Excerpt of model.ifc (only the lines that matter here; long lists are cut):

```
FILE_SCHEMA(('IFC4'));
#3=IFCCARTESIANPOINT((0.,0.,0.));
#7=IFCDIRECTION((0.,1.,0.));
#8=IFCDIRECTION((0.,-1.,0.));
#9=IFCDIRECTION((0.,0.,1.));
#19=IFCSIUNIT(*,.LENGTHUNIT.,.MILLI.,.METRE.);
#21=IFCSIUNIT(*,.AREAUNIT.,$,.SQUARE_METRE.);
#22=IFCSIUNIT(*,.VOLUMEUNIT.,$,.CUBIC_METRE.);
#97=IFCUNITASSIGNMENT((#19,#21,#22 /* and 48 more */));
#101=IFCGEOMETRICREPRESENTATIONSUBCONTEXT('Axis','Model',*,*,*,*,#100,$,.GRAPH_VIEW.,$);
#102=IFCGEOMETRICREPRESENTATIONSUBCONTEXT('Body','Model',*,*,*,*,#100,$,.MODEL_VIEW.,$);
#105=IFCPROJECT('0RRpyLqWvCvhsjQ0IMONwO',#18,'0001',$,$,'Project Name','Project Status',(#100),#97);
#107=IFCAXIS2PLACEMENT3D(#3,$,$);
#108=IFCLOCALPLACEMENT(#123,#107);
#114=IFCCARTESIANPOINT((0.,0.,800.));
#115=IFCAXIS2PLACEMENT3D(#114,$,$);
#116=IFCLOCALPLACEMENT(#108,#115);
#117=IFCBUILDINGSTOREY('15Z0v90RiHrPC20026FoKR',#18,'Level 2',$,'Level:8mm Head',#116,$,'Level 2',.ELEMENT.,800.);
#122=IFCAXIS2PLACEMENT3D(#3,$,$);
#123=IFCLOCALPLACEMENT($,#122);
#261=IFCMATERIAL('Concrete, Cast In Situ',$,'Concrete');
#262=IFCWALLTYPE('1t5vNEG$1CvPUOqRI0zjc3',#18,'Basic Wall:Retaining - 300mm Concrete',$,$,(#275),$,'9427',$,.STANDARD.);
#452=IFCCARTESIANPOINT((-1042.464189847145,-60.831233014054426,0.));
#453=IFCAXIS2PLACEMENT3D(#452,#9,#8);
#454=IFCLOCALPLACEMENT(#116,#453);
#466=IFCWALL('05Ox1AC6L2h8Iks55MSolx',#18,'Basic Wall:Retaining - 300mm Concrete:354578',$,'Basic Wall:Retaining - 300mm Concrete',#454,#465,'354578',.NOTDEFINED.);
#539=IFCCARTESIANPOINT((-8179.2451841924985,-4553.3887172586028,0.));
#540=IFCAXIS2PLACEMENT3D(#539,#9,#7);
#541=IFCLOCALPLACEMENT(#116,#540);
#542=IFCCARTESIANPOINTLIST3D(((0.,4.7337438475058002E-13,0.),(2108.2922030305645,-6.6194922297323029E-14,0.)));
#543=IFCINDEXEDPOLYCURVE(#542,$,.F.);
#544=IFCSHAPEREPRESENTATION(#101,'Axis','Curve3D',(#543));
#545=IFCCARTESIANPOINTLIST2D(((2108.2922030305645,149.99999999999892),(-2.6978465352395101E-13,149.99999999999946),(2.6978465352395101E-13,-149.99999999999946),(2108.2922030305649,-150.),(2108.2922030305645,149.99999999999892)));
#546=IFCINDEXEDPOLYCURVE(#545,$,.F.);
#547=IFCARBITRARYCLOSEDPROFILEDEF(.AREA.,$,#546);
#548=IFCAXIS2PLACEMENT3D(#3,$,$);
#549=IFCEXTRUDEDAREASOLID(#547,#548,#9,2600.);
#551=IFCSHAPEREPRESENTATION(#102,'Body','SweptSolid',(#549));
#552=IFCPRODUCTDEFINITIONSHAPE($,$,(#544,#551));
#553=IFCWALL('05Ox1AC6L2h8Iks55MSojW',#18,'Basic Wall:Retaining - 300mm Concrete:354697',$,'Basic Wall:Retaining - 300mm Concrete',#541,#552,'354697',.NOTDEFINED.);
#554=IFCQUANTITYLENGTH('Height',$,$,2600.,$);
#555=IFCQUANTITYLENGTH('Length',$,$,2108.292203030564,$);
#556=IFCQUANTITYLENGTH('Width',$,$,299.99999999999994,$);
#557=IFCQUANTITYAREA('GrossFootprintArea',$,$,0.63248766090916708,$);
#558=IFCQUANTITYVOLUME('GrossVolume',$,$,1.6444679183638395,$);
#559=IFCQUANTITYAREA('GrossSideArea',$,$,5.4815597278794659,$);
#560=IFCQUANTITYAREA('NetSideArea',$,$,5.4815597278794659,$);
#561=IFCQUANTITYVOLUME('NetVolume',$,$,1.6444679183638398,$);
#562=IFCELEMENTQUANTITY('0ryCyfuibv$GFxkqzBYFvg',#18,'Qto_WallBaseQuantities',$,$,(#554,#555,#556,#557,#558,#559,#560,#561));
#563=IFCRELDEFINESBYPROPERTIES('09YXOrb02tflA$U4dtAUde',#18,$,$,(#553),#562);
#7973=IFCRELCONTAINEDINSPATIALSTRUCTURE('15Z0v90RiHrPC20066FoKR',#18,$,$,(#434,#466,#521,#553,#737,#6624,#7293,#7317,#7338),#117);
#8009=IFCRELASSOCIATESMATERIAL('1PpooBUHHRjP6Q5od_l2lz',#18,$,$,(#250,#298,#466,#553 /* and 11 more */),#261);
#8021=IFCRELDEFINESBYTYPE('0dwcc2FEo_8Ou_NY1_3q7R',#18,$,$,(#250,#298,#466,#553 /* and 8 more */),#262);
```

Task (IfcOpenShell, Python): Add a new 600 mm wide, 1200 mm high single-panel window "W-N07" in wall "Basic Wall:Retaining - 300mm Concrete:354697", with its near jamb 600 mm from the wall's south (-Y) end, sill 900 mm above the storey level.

```python
import numpy as np
import ifcopenshell
import ifcopenshell.api.feature
import ifcopenshell.api.geometry
import ifcopenshell.api.pset
import ifcopenshell.api.root
import ifcopenshell.api.spatial
import ifcopenshell.geom
import ifcopenshell.util.element
import ifcopenshell.util.placement
import ifcopenshell.util.representation
import ifcopenshell.util.shape
import ifcopenshell.util.unit

model = ifcopenshell.open("model.ifc")
unit_scale = ifcopenshell.util.unit.calculate_unit_scale(model)
area_scale = ifcopenshell.util.unit.calculate_unit_scale(model, "AREAUNIT")
volume_scale = ifcopenshell.util.unit.calculate_unit_scale(model, "VOLUMEUNIT")
settings = ifcopenshell.geom.settings()


def volume(element):
    """Net volume in cubic metres, openings subtracted."""
    shape = ifcopenshell.geom.create_shape(settings, element)
    return ifcopenshell.util.shape.get_volume(shape.geometry)


wall = model.by_id(553)
storey = ifcopenshell.util.element.get_container(wall, ifc_class="IfcBuildingStorey")
context = ifcopenshell.util.representation.get_context(model, "Model", "Body", "MODEL_VIEW")
before = volume(wall)

width, height, from_end, sill = 0.6, 1.2, 0.6, 0.9  # metres

# The wall runs along its own X axis, and the end named is its -X end.
wall_shape = ifcopenshell.geom.create_shape(settings, wall)
x, y, z = ifcopenshell.util.shape.get_vertices(wall_shape.geometry).T
start = x.min() + from_end
face, thickness = float(y.min()), float(y.max() - y.min())
wall_matrix = ifcopenshell.util.placement.get_local_placement(wall.ObjectPlacement)
level = ifcopenshell.util.placement.get_local_placement(storey.ObjectPlacement)[2, 3]


def in_wall(x, y):
    """Placement at x, y metres in the wall's axes, at sill height."""
    matrix = wall_matrix.copy()
    matrix[:, 3] = wall_matrix @ np.array([x / unit_scale, y / unit_scale, 0.0, 1.0])
    matrix[2, 3] = level + sill / unit_scale
    return matrix


# Opening: a box that overshoots both wall faces by 50 mm.
opening = ifcopenshell.api.root.create_entity(model, ifc_class="IfcOpeningElement", predefined_type="OPENING")
box = ifcopenshell.api.geometry.add_wall_representation(
    model, context=context, length=width, height=height, thickness=thickness + 0.1
)
ifcopenshell.api.geometry.assign_representation(model, product=opening, representation=box)
ifcopenshell.api.geometry.edit_object_placement(model, product=opening, matrix=in_wall(start, face - 0.05), is_si=False)
ifcopenshell.api.feature.add_feature(model, feature=opening, element=wall)

window = ifcopenshell.api.root.create_entity(model, ifc_class="IfcWindow", name="W-N07", predefined_type="WINDOW")
window.OverallWidth, window.OverallHeight = width / unit_scale, height / unit_scale
window.PartitioningType = "SINGLE_PANEL"
body = ifcopenshell.api.geometry.add_window_representation(
    model,
    context=context,
    overall_width=window.OverallWidth,
    overall_height=window.OverallHeight,
    partition_type="SINGLE_PANEL",
)
ifcopenshell.api.geometry.assign_representation(model, product=window, representation=body)
ifcopenshell.api.spatial.assign_container(model, products=[window], relating_structure=storey)
ifcopenshell.api.feature.add_filling(model, opening=opening, element=window)

# Centre the window in the wall's thickness.
ifcopenshell.api.geometry.edit_object_placement(model, product=window, matrix=in_wall(start, face), is_si=False)
window_shape = ifcopenshell.geom.create_shape(settings, window)
depth = ifcopenshell.util.shape.get_vertices(window_shape.geometry)[:, 1]
offset = face + thickness / 2 - (depth.min() + depth.max()) / 2
ifcopenshell.api.geometry.edit_object_placement(model, product=window, matrix=in_wall(start, offset), is_si=False)

after = volume(wall)

# Update the wall's stored quantities.
qto = model.by_id(ifcopenshell.util.element.get_pset(wall, "Qto_WallBaseQuantities", should_inherit=False)["id"])
ifcopenshell.api.pset.edit_qto(model, qto=qto, properties={
    "NetSideArea": after / thickness / area_scale,
    "NetVolume": after / volume_scale,
})

print(f"wall volume {before:.3f} -> {after:.3f} m3")

model.write("model_v2.ifc")
```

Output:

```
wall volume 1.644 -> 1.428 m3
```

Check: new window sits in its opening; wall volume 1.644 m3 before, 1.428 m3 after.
